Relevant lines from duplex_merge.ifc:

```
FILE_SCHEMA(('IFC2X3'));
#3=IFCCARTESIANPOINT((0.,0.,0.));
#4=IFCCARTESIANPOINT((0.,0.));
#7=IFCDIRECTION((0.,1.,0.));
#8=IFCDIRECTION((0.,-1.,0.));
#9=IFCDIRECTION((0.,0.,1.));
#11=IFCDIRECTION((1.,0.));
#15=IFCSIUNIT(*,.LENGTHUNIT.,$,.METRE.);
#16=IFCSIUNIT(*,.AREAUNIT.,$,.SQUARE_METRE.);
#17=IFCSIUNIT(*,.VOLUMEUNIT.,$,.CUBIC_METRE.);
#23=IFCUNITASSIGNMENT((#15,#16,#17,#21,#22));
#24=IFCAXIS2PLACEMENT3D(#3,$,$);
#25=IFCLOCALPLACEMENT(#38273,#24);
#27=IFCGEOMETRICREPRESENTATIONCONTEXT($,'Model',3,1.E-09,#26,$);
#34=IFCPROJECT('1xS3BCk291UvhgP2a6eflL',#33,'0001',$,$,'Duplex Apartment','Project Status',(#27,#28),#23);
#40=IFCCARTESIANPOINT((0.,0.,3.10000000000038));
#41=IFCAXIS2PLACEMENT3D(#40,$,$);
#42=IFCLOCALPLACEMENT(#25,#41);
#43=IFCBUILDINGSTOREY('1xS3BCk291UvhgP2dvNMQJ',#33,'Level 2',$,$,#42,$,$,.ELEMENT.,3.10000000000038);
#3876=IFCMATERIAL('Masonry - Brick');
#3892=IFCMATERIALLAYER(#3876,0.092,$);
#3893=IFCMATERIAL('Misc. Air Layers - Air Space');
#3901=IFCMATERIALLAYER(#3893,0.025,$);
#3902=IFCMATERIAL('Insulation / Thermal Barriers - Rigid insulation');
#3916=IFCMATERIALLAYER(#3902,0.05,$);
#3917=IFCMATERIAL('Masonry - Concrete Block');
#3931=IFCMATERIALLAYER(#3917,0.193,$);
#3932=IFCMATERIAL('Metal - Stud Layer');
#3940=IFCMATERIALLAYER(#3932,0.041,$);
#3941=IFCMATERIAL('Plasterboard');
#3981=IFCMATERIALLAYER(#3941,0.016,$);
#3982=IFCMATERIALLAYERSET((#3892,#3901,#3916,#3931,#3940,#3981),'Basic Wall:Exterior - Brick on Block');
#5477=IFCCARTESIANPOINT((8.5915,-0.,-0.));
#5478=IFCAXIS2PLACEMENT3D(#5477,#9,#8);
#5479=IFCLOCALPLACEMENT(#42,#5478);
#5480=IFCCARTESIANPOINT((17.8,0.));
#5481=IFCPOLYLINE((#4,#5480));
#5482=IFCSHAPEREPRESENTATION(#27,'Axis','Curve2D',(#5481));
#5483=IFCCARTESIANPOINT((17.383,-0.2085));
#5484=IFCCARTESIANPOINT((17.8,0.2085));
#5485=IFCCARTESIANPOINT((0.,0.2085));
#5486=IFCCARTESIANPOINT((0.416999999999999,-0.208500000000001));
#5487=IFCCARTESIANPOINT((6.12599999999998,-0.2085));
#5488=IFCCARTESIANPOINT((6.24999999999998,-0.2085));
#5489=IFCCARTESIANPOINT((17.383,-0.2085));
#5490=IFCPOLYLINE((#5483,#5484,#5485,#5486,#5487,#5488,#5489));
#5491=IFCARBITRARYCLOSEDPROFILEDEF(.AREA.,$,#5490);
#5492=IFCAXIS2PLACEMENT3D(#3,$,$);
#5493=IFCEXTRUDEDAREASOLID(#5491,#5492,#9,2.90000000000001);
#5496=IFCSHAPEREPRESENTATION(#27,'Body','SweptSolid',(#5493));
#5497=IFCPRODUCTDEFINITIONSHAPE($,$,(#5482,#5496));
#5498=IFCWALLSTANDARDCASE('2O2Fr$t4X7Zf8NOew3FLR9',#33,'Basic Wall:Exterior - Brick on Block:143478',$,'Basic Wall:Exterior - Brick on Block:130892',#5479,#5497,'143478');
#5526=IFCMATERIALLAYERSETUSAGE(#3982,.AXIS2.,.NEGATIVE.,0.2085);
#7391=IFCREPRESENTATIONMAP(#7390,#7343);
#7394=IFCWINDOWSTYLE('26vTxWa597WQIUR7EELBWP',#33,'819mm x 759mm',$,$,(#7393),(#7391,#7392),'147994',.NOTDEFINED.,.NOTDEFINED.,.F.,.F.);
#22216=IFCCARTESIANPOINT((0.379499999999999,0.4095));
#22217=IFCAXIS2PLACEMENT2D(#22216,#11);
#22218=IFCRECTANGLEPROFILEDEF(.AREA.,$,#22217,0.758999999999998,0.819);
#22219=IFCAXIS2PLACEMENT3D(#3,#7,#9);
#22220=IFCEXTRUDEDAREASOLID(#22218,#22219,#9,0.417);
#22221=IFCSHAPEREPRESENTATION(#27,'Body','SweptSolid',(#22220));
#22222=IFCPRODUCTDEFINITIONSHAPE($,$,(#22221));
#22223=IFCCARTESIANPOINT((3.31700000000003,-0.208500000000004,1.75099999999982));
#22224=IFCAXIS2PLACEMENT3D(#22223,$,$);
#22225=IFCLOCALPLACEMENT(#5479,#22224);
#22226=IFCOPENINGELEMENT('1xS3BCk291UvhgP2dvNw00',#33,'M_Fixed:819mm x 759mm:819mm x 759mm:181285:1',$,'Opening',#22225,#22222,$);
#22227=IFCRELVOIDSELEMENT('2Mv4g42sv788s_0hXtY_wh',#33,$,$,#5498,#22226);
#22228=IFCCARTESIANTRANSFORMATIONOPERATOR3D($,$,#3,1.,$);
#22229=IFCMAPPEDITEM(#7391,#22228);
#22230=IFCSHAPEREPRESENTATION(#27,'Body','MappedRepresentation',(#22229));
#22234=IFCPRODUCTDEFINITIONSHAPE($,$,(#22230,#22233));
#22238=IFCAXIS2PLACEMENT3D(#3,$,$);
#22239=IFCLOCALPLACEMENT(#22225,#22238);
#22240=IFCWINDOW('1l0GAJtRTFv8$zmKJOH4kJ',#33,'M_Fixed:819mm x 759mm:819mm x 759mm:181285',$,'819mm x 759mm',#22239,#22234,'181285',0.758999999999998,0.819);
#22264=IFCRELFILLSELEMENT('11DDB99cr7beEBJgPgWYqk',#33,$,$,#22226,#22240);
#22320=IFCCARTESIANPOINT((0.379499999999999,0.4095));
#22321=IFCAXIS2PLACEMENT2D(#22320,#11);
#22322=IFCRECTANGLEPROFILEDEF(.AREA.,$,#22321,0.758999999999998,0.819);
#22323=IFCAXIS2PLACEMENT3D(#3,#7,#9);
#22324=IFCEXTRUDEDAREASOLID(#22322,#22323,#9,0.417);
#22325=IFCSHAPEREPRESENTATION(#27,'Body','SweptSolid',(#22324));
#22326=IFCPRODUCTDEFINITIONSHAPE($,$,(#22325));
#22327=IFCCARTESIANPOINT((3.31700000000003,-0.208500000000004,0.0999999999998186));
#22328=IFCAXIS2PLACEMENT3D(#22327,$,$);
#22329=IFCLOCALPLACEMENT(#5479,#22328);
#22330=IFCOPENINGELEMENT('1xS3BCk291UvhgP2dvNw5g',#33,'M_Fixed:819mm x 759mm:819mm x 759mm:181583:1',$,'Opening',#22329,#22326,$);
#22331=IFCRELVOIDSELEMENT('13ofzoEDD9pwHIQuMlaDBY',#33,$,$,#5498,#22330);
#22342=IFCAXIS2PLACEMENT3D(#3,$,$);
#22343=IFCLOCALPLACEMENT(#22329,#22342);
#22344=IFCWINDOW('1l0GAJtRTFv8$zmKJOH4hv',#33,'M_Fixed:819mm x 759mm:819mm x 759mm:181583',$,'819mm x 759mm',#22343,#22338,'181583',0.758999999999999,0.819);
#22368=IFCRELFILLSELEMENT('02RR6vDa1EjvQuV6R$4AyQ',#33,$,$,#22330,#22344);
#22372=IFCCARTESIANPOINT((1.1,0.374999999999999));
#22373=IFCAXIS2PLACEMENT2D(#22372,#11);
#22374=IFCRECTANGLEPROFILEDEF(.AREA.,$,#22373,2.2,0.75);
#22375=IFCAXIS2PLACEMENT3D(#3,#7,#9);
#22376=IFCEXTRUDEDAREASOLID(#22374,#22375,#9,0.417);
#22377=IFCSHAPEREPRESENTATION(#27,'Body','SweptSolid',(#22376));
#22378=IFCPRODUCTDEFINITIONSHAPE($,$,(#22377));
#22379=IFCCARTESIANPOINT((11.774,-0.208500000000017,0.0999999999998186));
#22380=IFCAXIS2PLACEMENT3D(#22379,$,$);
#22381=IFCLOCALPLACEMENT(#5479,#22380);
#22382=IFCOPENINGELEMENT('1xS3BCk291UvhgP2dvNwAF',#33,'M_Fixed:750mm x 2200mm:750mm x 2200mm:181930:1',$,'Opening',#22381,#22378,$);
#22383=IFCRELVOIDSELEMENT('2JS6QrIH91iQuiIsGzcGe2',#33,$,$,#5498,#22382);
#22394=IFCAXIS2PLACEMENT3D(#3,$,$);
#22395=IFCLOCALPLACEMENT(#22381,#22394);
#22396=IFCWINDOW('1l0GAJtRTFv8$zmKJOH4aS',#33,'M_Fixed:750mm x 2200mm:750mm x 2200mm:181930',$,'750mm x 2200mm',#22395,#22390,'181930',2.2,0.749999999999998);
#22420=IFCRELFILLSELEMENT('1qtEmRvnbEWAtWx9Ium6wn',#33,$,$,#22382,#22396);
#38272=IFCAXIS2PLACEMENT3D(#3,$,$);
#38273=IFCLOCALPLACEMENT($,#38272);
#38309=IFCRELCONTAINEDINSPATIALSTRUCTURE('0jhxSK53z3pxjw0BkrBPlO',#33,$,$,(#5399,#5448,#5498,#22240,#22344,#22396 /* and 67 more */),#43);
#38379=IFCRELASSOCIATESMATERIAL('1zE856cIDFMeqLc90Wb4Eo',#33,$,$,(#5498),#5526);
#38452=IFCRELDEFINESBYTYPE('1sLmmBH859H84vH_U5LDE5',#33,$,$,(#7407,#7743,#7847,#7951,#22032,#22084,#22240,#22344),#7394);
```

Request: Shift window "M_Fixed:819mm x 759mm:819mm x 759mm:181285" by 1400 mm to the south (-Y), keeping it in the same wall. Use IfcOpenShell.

```python
import ifcopenshell
import ifcopenshell.api.geometry
import ifcopenshell.util.placement
import ifcopenshell.util.unit

model = ifcopenshell.open("duplex_merge.ifc")
unit_scale = ifcopenshell.util.unit.calculate_unit_scale(model)

window = model.by_guid("1l0GAJtRTFv8$zmKJOH4kJ")
opening = window.FillsVoids[0].RelatingOpeningElement
wall = opening.VoidsElements[0].RelatingBuildingElement

wall_matrix = ifcopenshell.util.placement.get_local_placement(wall.ObjectPlacement)
shift = wall_matrix[:3, 0] * 1.4 / unit_scale
before = ifcopenshell.util.placement.get_local_placement(window.ObjectPlacement)[:3, 3].copy()

# The window is placed relative to its opening, so it follows when the opening moves.
matrix = ifcopenshell.util.placement.get_local_placement(opening.ObjectPlacement)
matrix[:3, 3] += shift
ifcopenshell.api.geometry.edit_object_placement(
    model, product=opening, matrix=matrix, is_si=False, should_transform_children=True
)

after = ifcopenshell.util.placement.get_local_placement(window.ObjectPlacement)[:3, 3]
print("window moved by", (after - before).round(3) + 0.0)

model.write("duplex_merge_v2.ifc")
```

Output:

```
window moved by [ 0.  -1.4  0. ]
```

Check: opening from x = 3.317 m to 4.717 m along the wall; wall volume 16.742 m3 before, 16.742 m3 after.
